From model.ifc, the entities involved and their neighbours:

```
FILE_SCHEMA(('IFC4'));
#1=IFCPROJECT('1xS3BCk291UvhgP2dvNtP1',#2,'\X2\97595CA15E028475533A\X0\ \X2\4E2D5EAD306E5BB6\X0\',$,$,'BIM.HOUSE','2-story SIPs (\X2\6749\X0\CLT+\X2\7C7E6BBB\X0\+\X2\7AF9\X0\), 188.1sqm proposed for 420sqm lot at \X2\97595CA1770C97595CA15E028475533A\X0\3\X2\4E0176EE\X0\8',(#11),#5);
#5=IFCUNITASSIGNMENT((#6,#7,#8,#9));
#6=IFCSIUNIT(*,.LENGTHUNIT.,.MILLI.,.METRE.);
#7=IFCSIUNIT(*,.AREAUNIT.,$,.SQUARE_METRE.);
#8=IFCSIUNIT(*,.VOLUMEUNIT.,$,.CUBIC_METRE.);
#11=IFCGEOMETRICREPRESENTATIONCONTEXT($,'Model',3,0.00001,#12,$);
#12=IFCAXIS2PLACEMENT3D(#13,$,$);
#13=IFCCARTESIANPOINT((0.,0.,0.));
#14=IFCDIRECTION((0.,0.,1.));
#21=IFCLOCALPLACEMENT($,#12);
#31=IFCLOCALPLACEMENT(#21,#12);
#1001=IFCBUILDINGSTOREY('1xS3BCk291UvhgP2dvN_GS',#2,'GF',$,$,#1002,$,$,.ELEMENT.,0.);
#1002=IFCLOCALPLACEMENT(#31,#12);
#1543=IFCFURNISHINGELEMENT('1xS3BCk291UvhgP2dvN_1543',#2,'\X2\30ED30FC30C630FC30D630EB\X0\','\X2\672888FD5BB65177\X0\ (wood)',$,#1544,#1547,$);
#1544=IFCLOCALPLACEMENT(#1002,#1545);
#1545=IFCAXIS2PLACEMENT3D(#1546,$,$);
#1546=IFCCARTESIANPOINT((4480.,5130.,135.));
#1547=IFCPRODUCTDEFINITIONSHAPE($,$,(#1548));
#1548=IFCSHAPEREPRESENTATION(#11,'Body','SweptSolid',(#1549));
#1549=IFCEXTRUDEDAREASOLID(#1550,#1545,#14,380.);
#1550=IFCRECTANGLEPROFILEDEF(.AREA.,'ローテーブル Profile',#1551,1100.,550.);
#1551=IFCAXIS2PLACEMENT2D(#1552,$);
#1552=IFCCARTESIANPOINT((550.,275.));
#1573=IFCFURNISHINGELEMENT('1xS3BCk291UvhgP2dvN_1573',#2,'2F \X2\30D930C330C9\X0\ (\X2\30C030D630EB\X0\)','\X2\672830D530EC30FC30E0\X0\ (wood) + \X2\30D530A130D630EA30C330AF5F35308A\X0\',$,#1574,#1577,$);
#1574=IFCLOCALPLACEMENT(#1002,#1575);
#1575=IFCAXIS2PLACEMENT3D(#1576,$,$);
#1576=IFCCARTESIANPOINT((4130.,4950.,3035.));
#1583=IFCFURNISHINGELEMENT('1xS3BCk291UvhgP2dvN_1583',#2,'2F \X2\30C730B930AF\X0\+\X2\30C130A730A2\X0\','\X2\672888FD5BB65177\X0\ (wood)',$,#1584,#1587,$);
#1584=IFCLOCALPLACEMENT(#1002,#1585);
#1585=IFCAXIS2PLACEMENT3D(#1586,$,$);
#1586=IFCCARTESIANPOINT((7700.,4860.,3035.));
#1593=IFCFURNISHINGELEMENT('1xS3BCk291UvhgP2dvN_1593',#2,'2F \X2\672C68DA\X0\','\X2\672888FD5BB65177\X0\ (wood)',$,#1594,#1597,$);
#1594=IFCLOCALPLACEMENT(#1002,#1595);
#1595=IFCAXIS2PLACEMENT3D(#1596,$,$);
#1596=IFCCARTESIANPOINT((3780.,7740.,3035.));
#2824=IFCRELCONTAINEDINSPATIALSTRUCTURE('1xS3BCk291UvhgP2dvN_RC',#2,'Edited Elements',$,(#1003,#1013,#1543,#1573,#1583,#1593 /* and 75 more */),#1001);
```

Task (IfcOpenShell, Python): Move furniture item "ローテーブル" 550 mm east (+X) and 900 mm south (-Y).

```python
import ifcopenshell
import ifcopenshell.api.geometry
import ifcopenshell.util.placement
import ifcopenshell.util.unit

model = ifcopenshell.open("model.ifc")
unit_scale = ifcopenshell.util.unit.calculate_unit_scale(model)

item = model.by_guid("1xS3BCk291UvhgP2dvN_1543")
matrix = ifcopenshell.util.placement.get_local_placement(item.ObjectPlacement)
matrix[0, 3] += 0.55 / unit_scale
matrix[1, 3] -= 0.9 / unit_scale
ifcopenshell.api.geometry.edit_object_placement(model, product=item, matrix=matrix, is_si=False)

print(ifcopenshell.util.placement.get_local_placement(item.ObjectPlacement).round(3) + 0.0)

model.write("model_rev.ifc")
```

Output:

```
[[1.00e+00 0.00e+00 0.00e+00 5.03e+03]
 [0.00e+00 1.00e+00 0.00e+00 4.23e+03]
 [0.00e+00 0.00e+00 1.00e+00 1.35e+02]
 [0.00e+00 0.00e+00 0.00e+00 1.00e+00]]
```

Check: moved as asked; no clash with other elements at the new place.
